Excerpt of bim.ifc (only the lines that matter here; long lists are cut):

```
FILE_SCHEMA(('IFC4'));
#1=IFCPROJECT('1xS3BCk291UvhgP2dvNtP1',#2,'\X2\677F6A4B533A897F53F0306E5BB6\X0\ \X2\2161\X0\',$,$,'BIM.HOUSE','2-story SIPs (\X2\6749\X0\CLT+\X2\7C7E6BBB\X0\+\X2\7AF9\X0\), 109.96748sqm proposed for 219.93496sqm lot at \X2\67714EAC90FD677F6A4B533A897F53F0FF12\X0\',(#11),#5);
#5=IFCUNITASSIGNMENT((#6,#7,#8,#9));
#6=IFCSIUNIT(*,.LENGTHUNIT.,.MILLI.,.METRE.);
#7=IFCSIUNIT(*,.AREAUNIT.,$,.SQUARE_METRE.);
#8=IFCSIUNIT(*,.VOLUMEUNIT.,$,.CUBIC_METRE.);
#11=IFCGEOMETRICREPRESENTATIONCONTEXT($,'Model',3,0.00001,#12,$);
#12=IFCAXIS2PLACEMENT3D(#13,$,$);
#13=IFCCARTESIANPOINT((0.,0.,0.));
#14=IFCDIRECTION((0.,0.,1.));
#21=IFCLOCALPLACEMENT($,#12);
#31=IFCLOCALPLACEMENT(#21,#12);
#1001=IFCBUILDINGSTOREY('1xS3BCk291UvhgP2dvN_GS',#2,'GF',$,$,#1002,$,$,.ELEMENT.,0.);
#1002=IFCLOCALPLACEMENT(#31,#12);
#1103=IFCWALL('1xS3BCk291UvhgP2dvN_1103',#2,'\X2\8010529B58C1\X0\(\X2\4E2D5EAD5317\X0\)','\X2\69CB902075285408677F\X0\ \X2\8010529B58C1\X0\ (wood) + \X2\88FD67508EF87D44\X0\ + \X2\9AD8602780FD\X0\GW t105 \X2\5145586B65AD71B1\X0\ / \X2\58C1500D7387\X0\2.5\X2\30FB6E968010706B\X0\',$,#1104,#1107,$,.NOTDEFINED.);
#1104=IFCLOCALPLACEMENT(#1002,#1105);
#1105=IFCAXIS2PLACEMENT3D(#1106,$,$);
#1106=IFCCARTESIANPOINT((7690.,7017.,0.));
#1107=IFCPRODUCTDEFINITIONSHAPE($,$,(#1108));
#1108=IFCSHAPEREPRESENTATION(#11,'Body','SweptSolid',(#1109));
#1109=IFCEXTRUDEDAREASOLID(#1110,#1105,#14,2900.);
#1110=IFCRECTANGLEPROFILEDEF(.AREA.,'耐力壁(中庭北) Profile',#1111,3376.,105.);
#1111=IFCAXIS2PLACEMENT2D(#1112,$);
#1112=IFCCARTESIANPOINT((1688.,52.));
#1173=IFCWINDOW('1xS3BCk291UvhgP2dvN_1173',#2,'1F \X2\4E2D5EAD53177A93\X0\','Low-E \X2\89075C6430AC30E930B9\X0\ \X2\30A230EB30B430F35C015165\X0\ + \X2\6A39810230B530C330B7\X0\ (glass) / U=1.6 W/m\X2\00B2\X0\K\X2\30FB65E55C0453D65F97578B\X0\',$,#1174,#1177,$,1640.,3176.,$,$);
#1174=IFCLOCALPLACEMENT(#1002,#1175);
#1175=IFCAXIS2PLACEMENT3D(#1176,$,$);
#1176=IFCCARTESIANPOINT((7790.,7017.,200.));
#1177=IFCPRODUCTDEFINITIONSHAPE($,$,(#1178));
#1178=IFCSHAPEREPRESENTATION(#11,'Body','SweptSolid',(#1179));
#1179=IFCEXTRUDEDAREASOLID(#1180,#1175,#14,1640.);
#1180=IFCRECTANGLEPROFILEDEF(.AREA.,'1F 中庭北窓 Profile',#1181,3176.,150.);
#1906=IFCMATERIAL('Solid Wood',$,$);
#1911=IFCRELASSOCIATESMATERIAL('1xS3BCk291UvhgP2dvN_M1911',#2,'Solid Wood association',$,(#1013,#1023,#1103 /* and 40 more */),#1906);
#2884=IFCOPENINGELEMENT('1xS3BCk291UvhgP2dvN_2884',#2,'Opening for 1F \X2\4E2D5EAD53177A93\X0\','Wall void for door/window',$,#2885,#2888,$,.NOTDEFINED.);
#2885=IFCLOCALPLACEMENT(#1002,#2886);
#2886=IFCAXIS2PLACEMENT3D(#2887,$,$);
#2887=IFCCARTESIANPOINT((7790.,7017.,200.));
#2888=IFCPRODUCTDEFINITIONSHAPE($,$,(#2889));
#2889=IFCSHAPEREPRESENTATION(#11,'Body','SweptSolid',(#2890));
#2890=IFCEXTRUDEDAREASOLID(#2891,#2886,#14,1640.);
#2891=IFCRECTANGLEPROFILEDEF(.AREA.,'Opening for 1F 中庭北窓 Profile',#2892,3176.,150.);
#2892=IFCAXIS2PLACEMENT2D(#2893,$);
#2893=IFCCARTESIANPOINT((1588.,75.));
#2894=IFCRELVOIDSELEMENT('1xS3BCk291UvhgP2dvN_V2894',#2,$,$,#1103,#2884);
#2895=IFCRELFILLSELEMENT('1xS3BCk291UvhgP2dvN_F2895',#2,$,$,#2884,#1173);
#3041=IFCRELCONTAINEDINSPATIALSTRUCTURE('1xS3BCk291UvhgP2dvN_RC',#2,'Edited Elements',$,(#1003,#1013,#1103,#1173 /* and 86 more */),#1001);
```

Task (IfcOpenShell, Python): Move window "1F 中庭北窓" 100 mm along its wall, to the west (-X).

```python
import ifcopenshell
import ifcopenshell.api.geometry
import ifcopenshell.util.placement
import ifcopenshell.util.unit

model = ifcopenshell.open("bim.ifc")
unit_scale = ifcopenshell.util.unit.calculate_unit_scale(model)

window = model.by_guid("1xS3BCk291UvhgP2dvN_1173")
opening = window.FillsVoids[0].RelatingOpeningElement
wall = opening.VoidsElements[0].RelatingBuildingElement

wall_matrix = ifcopenshell.util.placement.get_local_placement(wall.ObjectPlacement)
shift = wall_matrix[:3, 0] * -0.1 / unit_scale
before = ifcopenshell.util.placement.get_local_placement(window.ObjectPlacement)[:3, 3].copy()

# The window is not placed relative to its opening, so move both.
for product in (opening, window):
    matrix = ifcopenshell.util.placement.get_local_placement(product.ObjectPlacement)
    matrix[:3, 3] += shift
    ifcopenshell.api.geometry.edit_object_placement(model, product=product, matrix=matrix, is_si=False)

after = ifcopenshell.util.placement.get_local_placement(window.ObjectPlacement)[:3, 3]
print("window moved by", (after - before).round(3) + 0.0)

model.write("bim_v2.ifc")
```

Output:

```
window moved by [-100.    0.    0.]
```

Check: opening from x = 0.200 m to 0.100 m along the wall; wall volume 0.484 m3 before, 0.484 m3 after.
